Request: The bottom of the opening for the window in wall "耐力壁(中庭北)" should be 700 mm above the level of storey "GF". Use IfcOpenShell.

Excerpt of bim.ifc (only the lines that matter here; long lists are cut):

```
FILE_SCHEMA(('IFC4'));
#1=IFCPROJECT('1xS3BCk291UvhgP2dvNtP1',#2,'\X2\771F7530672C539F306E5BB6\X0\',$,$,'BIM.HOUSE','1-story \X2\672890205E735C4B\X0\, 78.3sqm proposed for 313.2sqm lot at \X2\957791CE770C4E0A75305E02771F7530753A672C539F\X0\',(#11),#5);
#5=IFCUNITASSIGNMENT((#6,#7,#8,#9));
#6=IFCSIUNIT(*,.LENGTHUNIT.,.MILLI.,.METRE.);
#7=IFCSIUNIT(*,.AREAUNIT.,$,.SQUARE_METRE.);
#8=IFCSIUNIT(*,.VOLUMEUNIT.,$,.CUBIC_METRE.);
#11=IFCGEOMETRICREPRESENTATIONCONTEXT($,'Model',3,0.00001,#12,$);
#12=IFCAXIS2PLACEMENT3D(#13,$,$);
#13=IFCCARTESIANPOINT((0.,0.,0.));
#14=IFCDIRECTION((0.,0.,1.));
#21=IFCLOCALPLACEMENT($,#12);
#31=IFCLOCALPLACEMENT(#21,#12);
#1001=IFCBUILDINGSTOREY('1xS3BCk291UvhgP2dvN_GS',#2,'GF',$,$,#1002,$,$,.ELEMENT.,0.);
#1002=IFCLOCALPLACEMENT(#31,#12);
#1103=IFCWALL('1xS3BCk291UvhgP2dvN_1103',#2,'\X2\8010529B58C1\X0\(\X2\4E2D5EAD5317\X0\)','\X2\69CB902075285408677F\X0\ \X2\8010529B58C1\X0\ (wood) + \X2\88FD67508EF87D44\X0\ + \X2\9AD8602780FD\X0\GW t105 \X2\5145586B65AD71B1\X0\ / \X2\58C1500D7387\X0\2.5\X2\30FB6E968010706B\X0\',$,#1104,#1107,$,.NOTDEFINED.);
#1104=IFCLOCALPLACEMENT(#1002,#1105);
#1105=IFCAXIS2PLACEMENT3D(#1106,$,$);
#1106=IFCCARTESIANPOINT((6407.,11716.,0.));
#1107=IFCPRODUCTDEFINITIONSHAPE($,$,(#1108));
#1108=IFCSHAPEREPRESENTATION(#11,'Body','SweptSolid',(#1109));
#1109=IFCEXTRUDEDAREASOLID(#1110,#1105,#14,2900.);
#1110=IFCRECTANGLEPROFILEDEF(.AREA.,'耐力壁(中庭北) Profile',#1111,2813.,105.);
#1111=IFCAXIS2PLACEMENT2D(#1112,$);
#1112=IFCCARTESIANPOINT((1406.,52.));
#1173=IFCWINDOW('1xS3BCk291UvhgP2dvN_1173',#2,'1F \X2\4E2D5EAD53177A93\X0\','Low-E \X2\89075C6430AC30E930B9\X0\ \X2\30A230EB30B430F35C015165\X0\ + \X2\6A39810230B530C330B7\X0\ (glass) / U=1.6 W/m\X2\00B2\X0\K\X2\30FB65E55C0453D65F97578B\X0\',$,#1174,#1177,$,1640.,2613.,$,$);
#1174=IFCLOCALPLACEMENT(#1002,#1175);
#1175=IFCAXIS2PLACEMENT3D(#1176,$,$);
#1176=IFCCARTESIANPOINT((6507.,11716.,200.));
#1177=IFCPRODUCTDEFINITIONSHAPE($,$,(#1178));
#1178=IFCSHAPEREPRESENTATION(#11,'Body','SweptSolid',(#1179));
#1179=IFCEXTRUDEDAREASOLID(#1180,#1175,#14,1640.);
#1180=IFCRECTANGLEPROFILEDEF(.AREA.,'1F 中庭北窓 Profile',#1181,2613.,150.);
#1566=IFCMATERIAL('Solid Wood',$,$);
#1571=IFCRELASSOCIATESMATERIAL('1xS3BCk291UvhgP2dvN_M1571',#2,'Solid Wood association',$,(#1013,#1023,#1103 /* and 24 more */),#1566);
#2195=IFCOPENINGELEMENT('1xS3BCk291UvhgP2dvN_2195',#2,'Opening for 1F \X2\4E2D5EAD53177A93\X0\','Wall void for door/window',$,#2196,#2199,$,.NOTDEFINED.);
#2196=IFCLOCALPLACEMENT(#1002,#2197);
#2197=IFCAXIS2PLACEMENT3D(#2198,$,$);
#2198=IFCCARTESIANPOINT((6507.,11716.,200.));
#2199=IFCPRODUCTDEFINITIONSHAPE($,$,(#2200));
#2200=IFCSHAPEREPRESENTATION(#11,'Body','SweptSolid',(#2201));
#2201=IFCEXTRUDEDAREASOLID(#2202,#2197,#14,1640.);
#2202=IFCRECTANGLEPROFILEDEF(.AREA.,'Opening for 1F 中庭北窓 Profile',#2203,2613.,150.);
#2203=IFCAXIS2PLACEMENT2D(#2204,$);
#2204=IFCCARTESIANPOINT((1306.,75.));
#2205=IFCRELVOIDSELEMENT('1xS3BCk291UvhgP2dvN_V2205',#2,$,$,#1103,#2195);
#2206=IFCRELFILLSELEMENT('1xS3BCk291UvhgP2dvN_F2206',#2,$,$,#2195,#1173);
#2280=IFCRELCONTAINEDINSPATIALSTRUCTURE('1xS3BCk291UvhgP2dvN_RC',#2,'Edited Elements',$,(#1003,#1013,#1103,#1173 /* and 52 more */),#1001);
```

```python
import numpy as np
import ifcopenshell
import ifcopenshell.api.geometry
import ifcopenshell.geom
import ifcopenshell.util.element
import ifcopenshell.util.placement
import ifcopenshell.util.shape
import ifcopenshell.util.unit

model = ifcopenshell.open("bim.ifc")
unit_scale = ifcopenshell.util.unit.calculate_unit_scale(model)

window = model.by_guid("1xS3BCk291UvhgP2dvN_1173")
opening = window.FillsVoids[0].RelatingOpeningElement
storey = ifcopenshell.util.element.get_container(window, ifc_class="IfcBuildingStorey")
level = ifcopenshell.util.placement.get_local_placement(storey.ObjectPlacement)[2, 3]

# The opening's origin need not be at the sill, so measure its lowest point.
shape = ifcopenshell.geom.create_shape(ifcopenshell.geom.settings(), opening)
bottom = ifcopenshell.util.shape.get_shape_bottom_elevation(shape, shape.geometry) / unit_scale
dz = level + 0.7 / unit_scale - bottom

shift = np.array([0.0, 0.0, dz])
# The window is not placed relative to its opening, so move both.
for product in (opening, window):
    matrix = ifcopenshell.util.placement.get_local_placement(product.ObjectPlacement)
    matrix[:3, 3] += shift
    ifcopenshell.api.geometry.edit_object_placement(model, product=product, matrix=matrix, is_si=False)

print(f"moved by {dz * unit_scale:+.3f} m")

model.write("bim_rev.ifc")
```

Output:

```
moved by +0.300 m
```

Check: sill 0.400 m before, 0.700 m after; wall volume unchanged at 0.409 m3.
